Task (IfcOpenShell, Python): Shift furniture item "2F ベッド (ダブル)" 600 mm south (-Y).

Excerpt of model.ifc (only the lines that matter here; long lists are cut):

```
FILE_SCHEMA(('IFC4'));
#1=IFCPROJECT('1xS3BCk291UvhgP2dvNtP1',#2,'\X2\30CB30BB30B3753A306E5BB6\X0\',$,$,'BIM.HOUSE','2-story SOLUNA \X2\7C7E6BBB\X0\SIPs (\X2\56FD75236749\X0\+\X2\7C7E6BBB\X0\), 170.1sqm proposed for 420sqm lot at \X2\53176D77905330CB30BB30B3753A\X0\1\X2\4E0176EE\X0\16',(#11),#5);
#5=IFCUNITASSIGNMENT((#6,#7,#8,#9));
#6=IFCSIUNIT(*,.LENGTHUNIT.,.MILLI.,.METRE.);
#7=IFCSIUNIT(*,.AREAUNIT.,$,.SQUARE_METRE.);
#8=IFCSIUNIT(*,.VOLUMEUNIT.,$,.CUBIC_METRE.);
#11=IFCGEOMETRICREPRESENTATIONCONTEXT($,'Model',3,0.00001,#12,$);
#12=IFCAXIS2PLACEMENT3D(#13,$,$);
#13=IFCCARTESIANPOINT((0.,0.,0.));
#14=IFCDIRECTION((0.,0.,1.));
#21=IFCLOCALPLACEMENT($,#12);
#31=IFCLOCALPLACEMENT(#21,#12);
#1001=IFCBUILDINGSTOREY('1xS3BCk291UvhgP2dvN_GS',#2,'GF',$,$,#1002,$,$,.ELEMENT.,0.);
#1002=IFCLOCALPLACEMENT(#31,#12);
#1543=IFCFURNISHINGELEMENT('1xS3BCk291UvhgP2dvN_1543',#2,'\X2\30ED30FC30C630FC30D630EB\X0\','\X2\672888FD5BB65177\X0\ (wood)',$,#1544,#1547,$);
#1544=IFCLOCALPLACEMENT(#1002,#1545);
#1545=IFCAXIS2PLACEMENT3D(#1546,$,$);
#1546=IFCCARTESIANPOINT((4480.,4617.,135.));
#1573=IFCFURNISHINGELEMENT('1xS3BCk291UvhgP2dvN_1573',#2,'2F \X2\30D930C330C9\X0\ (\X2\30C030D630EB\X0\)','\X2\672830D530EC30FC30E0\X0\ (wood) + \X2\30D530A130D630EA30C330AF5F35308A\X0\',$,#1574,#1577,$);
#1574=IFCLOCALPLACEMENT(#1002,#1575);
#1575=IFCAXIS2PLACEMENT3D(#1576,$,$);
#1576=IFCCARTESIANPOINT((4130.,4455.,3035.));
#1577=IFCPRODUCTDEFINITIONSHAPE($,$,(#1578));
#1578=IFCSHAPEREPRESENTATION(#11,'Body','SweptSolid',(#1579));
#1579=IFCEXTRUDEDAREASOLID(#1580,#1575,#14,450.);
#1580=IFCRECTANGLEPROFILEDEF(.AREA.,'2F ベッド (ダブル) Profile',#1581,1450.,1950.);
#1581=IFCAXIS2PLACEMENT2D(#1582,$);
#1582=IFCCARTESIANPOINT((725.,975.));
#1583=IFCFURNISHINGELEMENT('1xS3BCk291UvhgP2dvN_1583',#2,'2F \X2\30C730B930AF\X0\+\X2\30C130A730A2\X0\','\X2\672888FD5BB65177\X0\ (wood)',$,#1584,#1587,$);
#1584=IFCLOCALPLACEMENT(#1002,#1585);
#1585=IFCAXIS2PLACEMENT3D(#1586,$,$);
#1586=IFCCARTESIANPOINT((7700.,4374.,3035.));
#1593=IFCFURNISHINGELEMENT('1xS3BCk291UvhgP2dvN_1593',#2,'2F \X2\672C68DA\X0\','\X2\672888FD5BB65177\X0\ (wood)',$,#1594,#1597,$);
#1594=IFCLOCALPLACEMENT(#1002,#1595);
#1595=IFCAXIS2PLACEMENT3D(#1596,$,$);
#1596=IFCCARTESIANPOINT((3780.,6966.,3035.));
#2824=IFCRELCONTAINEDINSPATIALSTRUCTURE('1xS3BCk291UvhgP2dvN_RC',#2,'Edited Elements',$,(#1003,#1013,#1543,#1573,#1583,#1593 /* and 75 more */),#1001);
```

```python
import ifcopenshell
import ifcopenshell.api.geometry
import ifcopenshell.util.placement

model = ifcopenshell.open("model.ifc")

item = model.by_id(1573)
matrix = ifcopenshell.util.placement.get_local_placement(item.ObjectPlacement)
matrix[1, 3] -= 600.0
ifcopenshell.api.geometry.edit_object_placement(model, product=item, matrix=matrix, is_si=False)

print(ifcopenshell.util.placement.get_local_placement(item.ObjectPlacement).round(3) + 0.0)

model.write("model_updated.ifc")
```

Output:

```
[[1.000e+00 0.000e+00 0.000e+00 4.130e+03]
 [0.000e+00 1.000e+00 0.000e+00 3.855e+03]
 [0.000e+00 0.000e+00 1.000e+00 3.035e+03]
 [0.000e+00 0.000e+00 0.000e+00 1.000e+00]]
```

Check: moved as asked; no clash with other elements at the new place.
